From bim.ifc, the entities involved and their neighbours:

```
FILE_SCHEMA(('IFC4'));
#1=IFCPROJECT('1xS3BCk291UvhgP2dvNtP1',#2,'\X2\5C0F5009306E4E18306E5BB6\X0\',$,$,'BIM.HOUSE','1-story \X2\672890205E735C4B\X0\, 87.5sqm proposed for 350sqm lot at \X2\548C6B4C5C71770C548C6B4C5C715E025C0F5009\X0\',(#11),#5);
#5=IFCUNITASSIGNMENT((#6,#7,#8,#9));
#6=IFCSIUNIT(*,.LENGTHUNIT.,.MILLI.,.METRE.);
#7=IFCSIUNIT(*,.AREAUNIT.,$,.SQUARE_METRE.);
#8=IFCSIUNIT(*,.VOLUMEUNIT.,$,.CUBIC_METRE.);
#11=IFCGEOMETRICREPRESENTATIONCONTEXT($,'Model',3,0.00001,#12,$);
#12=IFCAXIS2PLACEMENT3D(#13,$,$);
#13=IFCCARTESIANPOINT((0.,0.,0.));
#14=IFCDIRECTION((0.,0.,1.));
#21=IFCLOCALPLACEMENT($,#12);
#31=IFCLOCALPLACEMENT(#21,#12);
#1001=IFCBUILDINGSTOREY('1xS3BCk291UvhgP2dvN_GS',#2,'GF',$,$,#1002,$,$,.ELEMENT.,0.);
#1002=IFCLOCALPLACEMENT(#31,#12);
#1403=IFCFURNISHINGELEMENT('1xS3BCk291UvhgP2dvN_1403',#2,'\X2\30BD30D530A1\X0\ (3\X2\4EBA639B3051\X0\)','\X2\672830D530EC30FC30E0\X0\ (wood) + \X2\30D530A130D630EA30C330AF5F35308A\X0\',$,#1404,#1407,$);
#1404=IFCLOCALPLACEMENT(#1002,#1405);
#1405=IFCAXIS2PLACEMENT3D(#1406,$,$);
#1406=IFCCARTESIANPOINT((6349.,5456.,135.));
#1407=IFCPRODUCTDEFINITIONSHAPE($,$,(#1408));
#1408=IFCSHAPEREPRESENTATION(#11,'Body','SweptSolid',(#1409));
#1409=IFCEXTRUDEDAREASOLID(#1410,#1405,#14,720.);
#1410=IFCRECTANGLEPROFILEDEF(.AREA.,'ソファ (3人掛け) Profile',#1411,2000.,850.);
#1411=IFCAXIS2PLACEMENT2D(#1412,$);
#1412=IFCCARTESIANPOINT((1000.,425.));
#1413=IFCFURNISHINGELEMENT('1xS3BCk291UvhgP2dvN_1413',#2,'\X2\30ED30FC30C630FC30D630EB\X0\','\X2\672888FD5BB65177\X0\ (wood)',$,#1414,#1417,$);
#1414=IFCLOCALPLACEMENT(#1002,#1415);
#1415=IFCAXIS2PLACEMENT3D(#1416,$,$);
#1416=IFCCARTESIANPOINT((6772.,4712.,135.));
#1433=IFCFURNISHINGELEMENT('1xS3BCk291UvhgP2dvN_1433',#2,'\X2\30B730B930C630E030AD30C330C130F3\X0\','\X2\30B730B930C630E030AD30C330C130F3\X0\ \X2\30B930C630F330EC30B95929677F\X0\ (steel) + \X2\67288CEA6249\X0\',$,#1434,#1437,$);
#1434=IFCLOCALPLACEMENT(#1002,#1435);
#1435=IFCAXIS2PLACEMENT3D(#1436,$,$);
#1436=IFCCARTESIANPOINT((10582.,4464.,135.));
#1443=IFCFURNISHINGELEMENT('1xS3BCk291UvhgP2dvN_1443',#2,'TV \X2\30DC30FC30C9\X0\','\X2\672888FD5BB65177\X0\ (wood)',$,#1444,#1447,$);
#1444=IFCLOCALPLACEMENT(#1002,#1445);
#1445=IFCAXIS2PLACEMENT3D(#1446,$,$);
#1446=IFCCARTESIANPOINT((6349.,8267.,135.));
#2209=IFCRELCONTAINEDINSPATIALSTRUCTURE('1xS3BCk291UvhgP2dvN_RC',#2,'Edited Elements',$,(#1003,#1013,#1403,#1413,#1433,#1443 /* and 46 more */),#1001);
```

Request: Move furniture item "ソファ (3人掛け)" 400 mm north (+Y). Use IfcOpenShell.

```python
import ifcopenshell
import ifcopenshell.api.geometry
import ifcopenshell.util.placement
import ifcopenshell.util.unit

model = ifcopenshell.open("bim.ifc")
unit_scale = ifcopenshell.util.unit.calculate_unit_scale(model)

item = model.by_guid("1xS3BCk291UvhgP2dvN_1403")
matrix = ifcopenshell.util.placement.get_local_placement(item.ObjectPlacement)
matrix[1, 3] += 0.4 / unit_scale
ifcopenshell.api.geometry.edit_object_placement(model, product=item, matrix=matrix, is_si=False)

print(ifcopenshell.util.placement.get_local_placement(item.ObjectPlacement).round(3) + 0.0)

model.write("bim-out.ifc")
```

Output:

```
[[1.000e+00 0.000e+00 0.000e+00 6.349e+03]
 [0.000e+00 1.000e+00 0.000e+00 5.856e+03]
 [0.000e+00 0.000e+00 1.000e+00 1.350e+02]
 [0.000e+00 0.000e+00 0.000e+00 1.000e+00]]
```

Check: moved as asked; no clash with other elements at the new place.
